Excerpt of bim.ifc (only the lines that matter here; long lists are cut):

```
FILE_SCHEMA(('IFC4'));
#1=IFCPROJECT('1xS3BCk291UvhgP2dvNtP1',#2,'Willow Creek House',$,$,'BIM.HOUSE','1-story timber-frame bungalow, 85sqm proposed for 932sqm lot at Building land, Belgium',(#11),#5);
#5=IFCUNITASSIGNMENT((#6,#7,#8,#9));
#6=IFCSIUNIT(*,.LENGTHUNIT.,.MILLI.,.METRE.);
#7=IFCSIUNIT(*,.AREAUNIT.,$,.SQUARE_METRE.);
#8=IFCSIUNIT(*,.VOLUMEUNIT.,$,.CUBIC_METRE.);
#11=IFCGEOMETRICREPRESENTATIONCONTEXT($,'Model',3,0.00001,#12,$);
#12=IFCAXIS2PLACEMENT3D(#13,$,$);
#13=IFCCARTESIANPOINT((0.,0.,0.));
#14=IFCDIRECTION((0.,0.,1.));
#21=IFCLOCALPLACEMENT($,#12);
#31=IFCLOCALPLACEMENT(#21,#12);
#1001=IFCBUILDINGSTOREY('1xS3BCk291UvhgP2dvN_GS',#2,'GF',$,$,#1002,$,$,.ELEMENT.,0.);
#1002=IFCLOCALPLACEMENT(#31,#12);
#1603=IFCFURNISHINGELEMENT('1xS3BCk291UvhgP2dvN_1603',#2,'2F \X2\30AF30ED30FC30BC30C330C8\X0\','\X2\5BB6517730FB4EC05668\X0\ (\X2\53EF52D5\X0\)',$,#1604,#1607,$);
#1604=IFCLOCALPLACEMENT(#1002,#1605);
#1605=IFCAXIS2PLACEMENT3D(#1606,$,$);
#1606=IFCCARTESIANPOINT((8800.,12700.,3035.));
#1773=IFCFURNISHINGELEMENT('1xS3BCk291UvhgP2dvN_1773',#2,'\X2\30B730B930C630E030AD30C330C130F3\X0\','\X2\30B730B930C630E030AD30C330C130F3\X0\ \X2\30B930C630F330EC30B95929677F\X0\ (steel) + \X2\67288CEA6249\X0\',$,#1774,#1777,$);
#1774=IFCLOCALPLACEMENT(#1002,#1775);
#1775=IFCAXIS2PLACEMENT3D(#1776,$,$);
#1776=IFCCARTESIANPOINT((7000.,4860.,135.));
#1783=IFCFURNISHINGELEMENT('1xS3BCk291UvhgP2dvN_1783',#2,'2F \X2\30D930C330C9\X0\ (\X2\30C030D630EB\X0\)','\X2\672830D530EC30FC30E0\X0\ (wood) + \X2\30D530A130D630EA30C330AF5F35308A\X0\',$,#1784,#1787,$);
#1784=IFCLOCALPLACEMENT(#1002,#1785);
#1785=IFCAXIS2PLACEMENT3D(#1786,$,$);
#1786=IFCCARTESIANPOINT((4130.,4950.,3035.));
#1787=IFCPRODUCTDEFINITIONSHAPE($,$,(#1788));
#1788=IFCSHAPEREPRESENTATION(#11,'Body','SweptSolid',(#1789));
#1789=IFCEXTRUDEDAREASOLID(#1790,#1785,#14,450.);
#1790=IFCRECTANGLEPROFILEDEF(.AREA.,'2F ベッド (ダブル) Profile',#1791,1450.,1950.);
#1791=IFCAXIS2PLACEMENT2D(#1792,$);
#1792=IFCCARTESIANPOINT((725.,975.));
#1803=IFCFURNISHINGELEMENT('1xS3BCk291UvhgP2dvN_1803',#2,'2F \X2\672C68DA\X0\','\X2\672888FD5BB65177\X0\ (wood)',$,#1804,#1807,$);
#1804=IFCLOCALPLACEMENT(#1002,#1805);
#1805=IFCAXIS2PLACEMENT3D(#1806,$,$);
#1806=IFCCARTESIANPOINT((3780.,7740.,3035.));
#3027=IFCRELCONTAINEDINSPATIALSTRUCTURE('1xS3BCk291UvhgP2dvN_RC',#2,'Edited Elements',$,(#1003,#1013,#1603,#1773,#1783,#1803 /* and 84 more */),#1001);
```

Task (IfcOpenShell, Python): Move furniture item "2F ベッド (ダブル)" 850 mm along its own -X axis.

```python
import ifcopenshell
import ifcopenshell.api.geometry
import ifcopenshell.util.placement
import ifcopenshell.util.unit

model = ifcopenshell.open("bim.ifc")
unit_scale = ifcopenshell.util.unit.calculate_unit_scale(model)

item = model.by_guid("1xS3BCk291UvhgP2dvN_1783")
matrix = ifcopenshell.util.placement.get_local_placement(item.ObjectPlacement)
matrix[:3, 3] -= matrix[:3, 0] * 0.85 / unit_scale
ifcopenshell.api.geometry.edit_object_placement(model, product=item, matrix=matrix, is_si=False)

print(ifcopenshell.util.placement.get_local_placement(item.ObjectPlacement).round(3) + 0.0)

model.write("bim_rev.ifc")
```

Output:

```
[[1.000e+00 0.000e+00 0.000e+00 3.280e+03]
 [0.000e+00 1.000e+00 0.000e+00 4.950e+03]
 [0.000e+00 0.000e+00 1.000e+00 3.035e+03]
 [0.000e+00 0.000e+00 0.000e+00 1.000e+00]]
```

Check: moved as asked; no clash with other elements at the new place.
